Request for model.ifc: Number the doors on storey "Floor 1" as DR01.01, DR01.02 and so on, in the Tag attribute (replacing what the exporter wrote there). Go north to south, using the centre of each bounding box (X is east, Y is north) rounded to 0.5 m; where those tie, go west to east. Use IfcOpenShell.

First a look at what the model holds.

```python
import ifcopenshell
import ifcopenshell.util.element
import ifcopenshell.util.placement

model = ifcopenshell.open("model.ifc")
print(model.schema)
storey = next(s for s in model.by_type("IfcBuildingStorey") if s.Name == "Floor 1")
doors = [e for e in ifcopenshell.util.element.get_decomposition(storey) if e.is_a("IfcDoor")]
for e in sorted(doors, key=lambda e: e.id()):
    origin = ifcopenshell.util.placement.get_local_placement(e.ObjectPlacement)[:3, 3]
    print(e.id(), e.Tag, e.Name, origin.round(2) + 0.0, sep=" | ")
```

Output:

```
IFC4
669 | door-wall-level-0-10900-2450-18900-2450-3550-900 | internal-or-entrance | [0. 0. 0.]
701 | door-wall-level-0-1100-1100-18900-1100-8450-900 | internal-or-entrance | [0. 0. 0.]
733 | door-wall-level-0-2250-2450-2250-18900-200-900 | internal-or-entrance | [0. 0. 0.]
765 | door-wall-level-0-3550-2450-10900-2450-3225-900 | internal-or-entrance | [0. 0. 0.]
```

```python
import ifcopenshell
import ifcopenshell.geom
import ifcopenshell.util.element
import ifcopenshell.util.shape

model = ifcopenshell.open("model.ifc")
settings = ifcopenshell.geom.settings()
settings.set("use-world-coords", True)


def centre(element):
    shape = ifcopenshell.geom.create_shape(settings, element)
    return ifcopenshell.util.shape.get_bbox_centroid(shape.geometry)


storey = next(s for s in model.by_type("IfcBuildingStorey") if s.Name == "Floor 1")
doors = [e for e in ifcopenshell.util.element.get_decomposition(storey) if e.is_a("IfcDoor")]

# Insertion points can sit at a corner or the storey origin, so sort by the geometry (in metres).
centres = {e: centre(e) for e in doors}
doors.sort(key=lambda e: (-round(centres[e][1] / 0.5), centres[e][0]))

for i, e in enumerate(doors, start=1):
    number = f"DR01.{i:02d}"
    e.Tag = number
    print(e.id(), number)

model.write("model_updated.ifc")
```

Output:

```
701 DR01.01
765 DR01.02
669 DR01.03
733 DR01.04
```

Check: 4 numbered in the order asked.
